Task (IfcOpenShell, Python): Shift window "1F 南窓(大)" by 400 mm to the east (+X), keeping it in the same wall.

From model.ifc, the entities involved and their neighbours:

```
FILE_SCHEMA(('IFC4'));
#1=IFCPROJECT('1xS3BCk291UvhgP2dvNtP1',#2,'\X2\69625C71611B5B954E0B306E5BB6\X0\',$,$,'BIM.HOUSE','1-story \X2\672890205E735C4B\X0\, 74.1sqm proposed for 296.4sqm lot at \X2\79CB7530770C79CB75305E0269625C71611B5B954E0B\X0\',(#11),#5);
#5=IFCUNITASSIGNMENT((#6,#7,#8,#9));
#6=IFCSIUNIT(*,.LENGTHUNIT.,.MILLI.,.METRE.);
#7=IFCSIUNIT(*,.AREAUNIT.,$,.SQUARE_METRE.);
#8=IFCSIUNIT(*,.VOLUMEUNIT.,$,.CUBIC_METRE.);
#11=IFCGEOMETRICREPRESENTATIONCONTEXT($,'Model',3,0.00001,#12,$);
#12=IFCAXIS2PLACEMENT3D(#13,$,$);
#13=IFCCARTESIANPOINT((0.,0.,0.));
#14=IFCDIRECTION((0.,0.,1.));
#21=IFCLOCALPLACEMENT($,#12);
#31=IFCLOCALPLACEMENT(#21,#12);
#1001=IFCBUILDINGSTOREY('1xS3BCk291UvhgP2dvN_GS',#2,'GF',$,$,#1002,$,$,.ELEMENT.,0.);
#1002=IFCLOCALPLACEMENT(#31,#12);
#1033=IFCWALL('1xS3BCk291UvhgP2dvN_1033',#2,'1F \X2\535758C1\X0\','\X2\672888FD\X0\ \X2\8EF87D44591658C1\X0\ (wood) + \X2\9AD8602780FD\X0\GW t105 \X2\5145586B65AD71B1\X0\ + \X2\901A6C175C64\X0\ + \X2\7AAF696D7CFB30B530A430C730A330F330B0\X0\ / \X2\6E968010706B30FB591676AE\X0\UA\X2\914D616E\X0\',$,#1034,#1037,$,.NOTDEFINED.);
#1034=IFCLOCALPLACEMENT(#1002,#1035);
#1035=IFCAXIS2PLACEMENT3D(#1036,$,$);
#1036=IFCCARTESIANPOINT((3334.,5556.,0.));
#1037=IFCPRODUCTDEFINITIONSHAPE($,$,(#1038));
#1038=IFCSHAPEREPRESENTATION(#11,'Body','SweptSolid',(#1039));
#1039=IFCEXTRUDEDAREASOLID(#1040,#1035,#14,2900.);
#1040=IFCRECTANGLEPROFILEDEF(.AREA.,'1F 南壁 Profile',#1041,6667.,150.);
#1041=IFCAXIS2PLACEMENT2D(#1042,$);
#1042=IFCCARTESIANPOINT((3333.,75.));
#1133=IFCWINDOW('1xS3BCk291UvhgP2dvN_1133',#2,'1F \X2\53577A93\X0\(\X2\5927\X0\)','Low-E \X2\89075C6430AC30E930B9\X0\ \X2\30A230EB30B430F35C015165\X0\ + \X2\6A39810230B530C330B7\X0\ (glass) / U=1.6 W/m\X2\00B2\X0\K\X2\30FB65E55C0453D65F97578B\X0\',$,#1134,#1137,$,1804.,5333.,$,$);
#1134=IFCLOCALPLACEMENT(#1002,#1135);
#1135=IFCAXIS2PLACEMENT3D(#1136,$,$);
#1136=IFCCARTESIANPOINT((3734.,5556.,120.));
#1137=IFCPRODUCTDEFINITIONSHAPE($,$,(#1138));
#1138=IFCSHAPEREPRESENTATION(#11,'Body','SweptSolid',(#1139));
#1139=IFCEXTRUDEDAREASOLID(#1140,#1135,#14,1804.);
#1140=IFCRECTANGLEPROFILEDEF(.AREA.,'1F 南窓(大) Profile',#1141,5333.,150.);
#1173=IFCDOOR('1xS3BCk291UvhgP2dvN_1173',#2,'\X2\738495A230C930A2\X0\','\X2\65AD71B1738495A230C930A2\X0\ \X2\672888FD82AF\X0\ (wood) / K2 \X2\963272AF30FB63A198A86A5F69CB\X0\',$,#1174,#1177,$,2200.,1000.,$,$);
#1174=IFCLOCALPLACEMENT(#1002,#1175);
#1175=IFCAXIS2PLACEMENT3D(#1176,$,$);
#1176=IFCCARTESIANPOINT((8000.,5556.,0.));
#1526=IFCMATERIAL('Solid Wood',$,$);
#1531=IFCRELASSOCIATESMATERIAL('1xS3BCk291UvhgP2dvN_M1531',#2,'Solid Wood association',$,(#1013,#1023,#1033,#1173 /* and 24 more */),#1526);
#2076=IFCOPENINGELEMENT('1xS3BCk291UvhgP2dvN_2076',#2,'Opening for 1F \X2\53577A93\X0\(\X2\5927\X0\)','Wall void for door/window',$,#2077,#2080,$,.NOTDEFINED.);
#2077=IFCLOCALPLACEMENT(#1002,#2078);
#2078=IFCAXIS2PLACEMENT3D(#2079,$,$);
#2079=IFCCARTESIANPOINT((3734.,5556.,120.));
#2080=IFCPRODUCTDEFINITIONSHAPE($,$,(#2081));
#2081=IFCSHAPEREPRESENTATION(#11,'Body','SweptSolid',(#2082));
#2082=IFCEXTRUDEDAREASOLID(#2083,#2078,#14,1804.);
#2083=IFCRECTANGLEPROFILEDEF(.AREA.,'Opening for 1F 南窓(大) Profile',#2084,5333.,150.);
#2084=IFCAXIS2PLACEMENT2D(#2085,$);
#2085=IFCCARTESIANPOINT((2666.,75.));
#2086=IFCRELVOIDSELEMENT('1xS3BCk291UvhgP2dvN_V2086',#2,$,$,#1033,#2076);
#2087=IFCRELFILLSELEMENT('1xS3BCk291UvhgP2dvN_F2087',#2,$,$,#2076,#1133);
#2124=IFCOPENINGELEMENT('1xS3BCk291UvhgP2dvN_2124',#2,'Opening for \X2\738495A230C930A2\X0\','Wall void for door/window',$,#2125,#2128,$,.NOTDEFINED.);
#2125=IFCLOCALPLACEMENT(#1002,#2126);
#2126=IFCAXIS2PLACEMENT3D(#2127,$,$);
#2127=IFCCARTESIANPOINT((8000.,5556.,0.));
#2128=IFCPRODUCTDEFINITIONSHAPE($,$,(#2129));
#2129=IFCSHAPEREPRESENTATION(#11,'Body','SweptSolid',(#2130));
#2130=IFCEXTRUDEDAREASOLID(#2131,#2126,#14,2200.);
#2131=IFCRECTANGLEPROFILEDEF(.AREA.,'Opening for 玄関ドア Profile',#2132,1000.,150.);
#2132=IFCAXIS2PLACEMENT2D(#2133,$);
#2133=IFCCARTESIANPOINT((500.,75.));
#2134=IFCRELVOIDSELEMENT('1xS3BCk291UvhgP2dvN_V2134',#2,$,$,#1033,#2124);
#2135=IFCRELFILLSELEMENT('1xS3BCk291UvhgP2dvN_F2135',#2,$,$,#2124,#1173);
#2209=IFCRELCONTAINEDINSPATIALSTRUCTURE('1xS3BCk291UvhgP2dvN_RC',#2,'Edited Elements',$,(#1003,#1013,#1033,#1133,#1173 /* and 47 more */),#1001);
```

```python
import ifcopenshell
import ifcopenshell.api.geometry
import ifcopenshell.util.placement
import ifcopenshell.util.unit

model = ifcopenshell.open("model.ifc")
unit_scale = ifcopenshell.util.unit.calculate_unit_scale(model)

window = model.by_guid("1xS3BCk291UvhgP2dvN_1133")
opening = window.FillsVoids[0].RelatingOpeningElement
wall = opening.VoidsElements[0].RelatingBuildingElement

wall_matrix = ifcopenshell.util.placement.get_local_placement(wall.ObjectPlacement)
shift = wall_matrix[:3, 0] * 0.4 / unit_scale
before = ifcopenshell.util.placement.get_local_placement(window.ObjectPlacement)[:3, 3].copy()

# The window is not placed relative to its opening, so move both.
for product in (opening, window):
    matrix = ifcopenshell.util.placement.get_local_placement(product.ObjectPlacement)
    matrix[:3, 3] += shift
    ifcopenshell.api.geometry.edit_object_placement(model, product=product, matrix=matrix, is_si=False)

after = ifcopenshell.util.placement.get_local_placement(window.ObjectPlacement)[:3, 3]
print("window moved by", (after - before).round(3) + 0.0)

model.write("model_rev.ifc")
```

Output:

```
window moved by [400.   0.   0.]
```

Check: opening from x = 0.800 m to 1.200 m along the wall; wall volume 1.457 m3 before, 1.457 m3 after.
